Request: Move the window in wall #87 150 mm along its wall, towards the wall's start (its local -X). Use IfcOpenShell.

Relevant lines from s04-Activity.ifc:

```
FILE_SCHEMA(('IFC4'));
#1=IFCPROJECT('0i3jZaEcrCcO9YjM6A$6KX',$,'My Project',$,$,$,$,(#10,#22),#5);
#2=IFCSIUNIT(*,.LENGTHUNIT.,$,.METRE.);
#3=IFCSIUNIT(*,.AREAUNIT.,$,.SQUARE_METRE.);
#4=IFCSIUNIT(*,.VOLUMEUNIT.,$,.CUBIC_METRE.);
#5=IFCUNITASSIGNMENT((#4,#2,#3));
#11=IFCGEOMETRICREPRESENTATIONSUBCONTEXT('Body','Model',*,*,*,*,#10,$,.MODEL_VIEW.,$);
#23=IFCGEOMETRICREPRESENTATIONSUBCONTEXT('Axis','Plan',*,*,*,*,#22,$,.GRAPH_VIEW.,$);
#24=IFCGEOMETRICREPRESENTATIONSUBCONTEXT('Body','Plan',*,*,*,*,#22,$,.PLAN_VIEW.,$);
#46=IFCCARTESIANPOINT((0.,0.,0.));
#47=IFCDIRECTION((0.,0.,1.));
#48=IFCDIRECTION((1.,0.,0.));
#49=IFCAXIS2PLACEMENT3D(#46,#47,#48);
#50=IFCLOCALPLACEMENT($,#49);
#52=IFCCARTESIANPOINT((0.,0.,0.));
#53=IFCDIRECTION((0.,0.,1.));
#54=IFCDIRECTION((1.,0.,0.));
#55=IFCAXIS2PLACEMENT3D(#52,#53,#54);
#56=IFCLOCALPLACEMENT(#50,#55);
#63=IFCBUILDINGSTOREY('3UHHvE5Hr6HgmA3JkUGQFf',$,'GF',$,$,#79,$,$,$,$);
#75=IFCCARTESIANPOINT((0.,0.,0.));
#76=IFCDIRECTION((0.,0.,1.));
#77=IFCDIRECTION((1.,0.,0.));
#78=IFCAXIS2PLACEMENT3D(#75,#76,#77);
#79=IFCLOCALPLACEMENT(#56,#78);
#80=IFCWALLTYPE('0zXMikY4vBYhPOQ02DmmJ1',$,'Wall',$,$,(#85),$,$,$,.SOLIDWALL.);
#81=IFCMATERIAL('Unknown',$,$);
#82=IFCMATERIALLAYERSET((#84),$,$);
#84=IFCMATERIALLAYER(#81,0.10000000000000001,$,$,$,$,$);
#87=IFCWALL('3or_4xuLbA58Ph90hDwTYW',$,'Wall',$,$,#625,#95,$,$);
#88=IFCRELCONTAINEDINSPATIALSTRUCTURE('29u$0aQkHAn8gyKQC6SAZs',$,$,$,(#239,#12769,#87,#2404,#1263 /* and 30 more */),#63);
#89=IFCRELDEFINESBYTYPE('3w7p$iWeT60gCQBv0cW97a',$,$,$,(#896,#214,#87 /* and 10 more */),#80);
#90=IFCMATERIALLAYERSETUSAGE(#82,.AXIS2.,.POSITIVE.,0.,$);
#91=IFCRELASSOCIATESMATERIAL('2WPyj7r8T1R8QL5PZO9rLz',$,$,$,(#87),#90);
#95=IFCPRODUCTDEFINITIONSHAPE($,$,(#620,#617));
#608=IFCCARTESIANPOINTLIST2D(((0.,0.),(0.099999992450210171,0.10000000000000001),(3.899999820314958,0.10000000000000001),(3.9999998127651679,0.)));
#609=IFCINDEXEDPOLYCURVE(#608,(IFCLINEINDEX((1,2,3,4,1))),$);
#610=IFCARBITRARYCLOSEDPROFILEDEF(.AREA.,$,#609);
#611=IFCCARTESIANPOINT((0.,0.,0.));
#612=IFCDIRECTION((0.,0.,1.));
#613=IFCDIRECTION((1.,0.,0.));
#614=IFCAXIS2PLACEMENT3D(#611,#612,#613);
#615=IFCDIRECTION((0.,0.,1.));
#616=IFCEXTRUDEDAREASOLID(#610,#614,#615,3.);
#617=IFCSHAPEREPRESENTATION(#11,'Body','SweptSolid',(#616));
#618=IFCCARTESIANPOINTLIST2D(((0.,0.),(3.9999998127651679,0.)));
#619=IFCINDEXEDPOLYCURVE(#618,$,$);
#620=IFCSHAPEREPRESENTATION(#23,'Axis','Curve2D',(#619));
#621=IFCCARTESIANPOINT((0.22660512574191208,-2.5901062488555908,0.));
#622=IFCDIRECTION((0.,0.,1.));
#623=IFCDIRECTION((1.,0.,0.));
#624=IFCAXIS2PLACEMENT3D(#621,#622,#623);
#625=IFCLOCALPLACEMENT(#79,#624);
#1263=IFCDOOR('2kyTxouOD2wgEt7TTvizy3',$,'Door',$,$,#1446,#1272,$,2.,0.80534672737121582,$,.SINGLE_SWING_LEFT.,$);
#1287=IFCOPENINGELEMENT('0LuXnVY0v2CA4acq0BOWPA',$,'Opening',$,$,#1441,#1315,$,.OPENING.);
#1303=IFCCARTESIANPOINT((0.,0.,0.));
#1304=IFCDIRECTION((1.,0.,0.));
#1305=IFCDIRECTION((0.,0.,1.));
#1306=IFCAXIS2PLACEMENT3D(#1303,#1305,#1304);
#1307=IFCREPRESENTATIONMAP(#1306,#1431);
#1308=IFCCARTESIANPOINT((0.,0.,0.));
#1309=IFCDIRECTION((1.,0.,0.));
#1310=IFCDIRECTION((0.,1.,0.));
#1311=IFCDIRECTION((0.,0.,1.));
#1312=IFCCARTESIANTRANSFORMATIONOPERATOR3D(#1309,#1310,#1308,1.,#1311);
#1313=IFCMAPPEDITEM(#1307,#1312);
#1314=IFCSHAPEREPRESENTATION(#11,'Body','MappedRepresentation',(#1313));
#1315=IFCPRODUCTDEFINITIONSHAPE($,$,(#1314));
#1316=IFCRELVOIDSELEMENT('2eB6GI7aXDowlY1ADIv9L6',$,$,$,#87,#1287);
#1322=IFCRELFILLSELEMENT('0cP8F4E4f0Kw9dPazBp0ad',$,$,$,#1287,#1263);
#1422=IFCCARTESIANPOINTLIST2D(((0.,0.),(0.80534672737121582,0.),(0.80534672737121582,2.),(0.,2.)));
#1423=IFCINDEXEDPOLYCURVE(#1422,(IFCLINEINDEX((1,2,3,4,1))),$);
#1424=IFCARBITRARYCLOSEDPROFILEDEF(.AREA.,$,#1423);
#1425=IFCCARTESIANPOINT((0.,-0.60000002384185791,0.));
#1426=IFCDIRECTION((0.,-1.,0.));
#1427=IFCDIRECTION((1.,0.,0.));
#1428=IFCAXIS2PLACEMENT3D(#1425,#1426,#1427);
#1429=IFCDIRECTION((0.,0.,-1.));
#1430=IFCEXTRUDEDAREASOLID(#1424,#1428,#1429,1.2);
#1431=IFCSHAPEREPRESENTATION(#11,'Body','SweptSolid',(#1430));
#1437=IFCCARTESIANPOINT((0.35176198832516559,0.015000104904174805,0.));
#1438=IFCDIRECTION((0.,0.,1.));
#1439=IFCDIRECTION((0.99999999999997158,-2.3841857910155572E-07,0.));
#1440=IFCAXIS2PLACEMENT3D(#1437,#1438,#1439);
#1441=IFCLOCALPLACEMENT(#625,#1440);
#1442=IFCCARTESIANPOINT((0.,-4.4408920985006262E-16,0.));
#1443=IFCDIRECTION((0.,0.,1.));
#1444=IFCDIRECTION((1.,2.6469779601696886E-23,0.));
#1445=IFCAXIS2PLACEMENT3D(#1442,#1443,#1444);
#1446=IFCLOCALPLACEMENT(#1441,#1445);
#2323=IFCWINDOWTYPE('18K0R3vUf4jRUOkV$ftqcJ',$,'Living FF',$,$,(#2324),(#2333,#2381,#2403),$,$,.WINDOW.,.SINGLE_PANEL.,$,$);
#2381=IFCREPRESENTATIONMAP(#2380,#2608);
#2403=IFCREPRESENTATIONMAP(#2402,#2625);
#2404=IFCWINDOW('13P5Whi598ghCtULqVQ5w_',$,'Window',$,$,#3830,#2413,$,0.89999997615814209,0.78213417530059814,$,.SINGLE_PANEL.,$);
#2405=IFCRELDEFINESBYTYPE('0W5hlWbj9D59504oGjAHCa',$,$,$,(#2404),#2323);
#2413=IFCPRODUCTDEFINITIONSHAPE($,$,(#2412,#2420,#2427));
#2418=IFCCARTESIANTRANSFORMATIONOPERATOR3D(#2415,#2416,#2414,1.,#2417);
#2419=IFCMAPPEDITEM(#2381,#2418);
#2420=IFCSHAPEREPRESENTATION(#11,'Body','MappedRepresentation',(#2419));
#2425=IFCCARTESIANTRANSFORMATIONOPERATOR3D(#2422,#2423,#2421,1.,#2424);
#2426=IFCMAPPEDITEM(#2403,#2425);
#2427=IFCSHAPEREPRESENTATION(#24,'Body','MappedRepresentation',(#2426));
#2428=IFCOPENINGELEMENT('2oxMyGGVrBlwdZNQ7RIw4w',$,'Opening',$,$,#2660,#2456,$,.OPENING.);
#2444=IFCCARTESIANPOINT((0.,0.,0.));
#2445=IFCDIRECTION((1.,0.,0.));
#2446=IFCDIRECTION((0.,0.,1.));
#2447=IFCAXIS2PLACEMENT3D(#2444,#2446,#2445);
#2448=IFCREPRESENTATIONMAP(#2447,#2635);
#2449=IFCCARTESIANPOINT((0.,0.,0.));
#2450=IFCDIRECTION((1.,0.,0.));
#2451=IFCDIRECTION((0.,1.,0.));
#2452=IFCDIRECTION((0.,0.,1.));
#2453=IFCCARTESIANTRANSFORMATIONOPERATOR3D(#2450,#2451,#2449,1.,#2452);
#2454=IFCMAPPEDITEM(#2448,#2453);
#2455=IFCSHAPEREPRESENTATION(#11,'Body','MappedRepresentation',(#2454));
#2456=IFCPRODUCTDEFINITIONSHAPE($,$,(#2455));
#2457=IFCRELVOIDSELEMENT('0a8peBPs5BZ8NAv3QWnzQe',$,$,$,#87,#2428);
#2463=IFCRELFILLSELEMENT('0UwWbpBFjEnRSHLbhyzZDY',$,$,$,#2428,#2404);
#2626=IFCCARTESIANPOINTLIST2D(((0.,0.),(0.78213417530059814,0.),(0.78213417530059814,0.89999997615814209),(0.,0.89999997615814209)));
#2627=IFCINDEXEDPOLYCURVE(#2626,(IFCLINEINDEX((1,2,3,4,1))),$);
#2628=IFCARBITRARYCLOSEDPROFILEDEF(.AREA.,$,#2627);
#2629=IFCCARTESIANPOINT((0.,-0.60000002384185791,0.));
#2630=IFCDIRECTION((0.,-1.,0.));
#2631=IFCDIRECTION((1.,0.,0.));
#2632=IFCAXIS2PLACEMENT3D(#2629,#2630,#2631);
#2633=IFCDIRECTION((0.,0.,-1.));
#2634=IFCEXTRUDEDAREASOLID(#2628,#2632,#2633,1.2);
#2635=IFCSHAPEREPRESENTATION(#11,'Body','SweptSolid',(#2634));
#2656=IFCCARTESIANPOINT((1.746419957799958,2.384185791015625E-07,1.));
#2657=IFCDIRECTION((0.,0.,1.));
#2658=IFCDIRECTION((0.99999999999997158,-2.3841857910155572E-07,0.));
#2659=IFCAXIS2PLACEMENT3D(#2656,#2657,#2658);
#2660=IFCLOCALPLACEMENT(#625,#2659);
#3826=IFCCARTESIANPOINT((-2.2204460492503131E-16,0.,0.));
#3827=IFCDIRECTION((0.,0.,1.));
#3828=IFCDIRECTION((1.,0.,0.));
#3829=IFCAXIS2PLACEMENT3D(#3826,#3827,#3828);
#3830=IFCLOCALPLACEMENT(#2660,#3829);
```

```python
import ifcopenshell
import ifcopenshell.api.geometry
import ifcopenshell.util.placement
import ifcopenshell.util.unit

model = ifcopenshell.open("s04-Activity.ifc")
unit_scale = ifcopenshell.util.unit.calculate_unit_scale(model)

window = model.by_id(2404)
opening = window.FillsVoids[0].RelatingOpeningElement
wall = opening.VoidsElements[0].RelatingBuildingElement

wall_matrix = ifcopenshell.util.placement.get_local_placement(wall.ObjectPlacement)
shift = wall_matrix[:3, 0] * -0.15 / unit_scale
before = ifcopenshell.util.placement.get_local_placement(window.ObjectPlacement)[:3, 3].copy()

# The window is placed relative to its opening, so it follows when the opening moves.
matrix = ifcopenshell.util.placement.get_local_placement(opening.ObjectPlacement)
matrix[:3, 3] += shift
ifcopenshell.api.geometry.edit_object_placement(
    model, product=opening, matrix=matrix, is_si=False, should_transform_children=True
)

after = ifcopenshell.util.placement.get_local_placement(window.ObjectPlacement)[:3, 3]
print("window moved by", (after - before).round(3) + 0.0)

model.write("s04-Activity_updated.ifc")
```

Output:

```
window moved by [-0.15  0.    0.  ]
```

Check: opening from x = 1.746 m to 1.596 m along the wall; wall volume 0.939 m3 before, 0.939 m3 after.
